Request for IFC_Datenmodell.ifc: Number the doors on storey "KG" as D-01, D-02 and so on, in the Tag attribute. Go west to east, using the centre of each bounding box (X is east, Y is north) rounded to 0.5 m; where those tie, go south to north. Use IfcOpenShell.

First a look at what the model holds.

```python
import ifcopenshell
import ifcopenshell.util.element
import ifcopenshell.util.placement

model = ifcopenshell.open("IFC_Datenmodell.ifc")
print(model.schema)
storey = next(s for s in model.by_type("IfcBuildingStorey") if s.Name == "KG")
doors = [e for e in ifcopenshell.util.element.get_decomposition(storey) if e.is_a("IfcDoor")]
for e in sorted(doors, key=lambda e: e.id()):
    origin = ifcopenshell.util.placement.get_local_placement(e.ObjectPlacement)[:3, 3]
    print(e.id(), e.Tag, e.Name, origin.round(2) + 0.0, sep=" | ")
```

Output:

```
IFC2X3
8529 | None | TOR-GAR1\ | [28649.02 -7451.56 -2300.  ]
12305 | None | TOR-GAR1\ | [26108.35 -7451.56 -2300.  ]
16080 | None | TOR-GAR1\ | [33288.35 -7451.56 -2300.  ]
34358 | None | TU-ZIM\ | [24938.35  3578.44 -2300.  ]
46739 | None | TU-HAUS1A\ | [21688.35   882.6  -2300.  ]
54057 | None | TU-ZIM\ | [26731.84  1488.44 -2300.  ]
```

```python
import ifcopenshell
import ifcopenshell.geom
import ifcopenshell.util.element
import ifcopenshell.util.shape

model = ifcopenshell.open("IFC_Datenmodell.ifc")
settings = ifcopenshell.geom.settings()
settings.set("use-world-coords", True)


def centre(element):
    shape = ifcopenshell.geom.create_shape(settings, element)
    return ifcopenshell.util.shape.get_bbox_centroid(shape.geometry)


storey = next(s for s in model.by_type("IfcBuildingStorey") if s.Name == "KG")
doors = [e for e in ifcopenshell.util.element.get_decomposition(storey) if e.is_a("IfcDoor")]

# Insertion points can sit at a corner or the storey origin, so sort by the geometry (in metres).
centres = {e: centre(e) for e in doors}
doors.sort(key=lambda e: (round(centres[e][0] / 0.5), centres[e][1]))

for i, e in enumerate(doors, start=1):
    number = f"D-{i:02d}"
    e.Tag = number
    print(e.id(), number)

model.write("IFC_Datenmodell-out.ifc")
```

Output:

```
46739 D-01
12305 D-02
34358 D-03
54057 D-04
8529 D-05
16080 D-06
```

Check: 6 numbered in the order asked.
